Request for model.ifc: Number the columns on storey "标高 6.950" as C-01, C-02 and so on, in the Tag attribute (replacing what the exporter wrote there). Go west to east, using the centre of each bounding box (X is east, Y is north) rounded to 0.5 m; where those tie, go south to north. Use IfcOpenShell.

First a look at what the model holds.

```python
import ifcopenshell
import ifcopenshell.util.element
import ifcopenshell.util.placement

model = ifcopenshell.open("model.ifc")
print(model.schema)
storey = next(s for s in model.by_type("IfcBuildingStorey") if s.Name == "标高 6.950")
columns = [e for e in ifcopenshell.util.element.get_decomposition(storey) if e.is_a("IfcColumn")]
for e in sorted(columns, key=lambda e: e.id()):
    origin = ifcopenshell.util.placement.get_local_placement(e.ObjectPlacement)[:3, 3]
    print(e.id(), e.Tag, e.Name, origin.round(2) + 0.0, sep=" | ")
```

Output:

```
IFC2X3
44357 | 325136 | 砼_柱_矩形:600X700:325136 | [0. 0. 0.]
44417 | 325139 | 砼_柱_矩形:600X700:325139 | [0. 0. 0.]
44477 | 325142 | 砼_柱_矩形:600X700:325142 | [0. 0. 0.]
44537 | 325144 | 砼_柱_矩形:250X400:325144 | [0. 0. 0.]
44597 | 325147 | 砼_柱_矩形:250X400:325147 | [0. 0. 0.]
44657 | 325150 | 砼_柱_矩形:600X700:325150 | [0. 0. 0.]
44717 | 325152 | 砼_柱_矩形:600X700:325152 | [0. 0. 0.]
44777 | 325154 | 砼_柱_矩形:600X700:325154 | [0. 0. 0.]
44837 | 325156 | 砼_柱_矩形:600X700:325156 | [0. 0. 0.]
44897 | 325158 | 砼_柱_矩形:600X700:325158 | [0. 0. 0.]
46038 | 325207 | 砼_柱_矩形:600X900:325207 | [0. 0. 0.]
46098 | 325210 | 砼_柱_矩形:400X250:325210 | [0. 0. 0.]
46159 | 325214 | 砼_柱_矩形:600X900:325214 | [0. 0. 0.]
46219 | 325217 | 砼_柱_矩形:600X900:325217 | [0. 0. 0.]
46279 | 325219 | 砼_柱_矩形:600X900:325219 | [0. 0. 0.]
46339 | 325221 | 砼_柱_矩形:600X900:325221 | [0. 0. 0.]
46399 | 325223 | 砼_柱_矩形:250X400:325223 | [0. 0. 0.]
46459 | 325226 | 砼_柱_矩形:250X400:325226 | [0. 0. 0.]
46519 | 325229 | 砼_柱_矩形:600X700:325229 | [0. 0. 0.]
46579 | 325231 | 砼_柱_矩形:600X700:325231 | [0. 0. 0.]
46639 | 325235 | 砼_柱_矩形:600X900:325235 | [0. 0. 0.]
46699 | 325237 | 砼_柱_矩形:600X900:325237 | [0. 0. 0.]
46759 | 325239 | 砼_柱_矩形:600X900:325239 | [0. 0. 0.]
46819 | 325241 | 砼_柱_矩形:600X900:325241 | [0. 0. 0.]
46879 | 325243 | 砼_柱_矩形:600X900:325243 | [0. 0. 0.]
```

```python
import ifcopenshell
import ifcopenshell.geom
import ifcopenshell.util.element
import ifcopenshell.util.shape

model = ifcopenshell.open("model.ifc")
settings = ifcopenshell.geom.settings()
settings.set("use-world-coords", True)


def centre(element):
    shape = ifcopenshell.geom.create_shape(settings, element)
    return ifcopenshell.util.shape.get_bbox_centroid(shape.geometry)


storey = next(s for s in model.by_type("IfcBuildingStorey") if s.Name == "标高 6.950")
columns = [e for e in ifcopenshell.util.element.get_decomposition(storey) if e.is_a("IfcColumn")]

# Insertion points can sit at a corner or the storey origin, so sort by the geometry (in metres).
centres = {e: centre(e) for e in columns}
columns.sort(key=lambda e: (round(centres[e][0] / 0.5), centres[e][1]))

for i, e in enumerate(columns, start=1):
    number = f"C-{i:02d}"
    e.Tag = number
    print(e.id(), number)

model.write("model_updated.ifc")
```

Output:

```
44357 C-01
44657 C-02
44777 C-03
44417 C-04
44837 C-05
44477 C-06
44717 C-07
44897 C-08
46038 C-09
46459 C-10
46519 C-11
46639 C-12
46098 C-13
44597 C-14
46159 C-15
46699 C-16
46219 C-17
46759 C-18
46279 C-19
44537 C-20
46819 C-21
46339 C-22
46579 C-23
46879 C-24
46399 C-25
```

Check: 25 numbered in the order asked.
